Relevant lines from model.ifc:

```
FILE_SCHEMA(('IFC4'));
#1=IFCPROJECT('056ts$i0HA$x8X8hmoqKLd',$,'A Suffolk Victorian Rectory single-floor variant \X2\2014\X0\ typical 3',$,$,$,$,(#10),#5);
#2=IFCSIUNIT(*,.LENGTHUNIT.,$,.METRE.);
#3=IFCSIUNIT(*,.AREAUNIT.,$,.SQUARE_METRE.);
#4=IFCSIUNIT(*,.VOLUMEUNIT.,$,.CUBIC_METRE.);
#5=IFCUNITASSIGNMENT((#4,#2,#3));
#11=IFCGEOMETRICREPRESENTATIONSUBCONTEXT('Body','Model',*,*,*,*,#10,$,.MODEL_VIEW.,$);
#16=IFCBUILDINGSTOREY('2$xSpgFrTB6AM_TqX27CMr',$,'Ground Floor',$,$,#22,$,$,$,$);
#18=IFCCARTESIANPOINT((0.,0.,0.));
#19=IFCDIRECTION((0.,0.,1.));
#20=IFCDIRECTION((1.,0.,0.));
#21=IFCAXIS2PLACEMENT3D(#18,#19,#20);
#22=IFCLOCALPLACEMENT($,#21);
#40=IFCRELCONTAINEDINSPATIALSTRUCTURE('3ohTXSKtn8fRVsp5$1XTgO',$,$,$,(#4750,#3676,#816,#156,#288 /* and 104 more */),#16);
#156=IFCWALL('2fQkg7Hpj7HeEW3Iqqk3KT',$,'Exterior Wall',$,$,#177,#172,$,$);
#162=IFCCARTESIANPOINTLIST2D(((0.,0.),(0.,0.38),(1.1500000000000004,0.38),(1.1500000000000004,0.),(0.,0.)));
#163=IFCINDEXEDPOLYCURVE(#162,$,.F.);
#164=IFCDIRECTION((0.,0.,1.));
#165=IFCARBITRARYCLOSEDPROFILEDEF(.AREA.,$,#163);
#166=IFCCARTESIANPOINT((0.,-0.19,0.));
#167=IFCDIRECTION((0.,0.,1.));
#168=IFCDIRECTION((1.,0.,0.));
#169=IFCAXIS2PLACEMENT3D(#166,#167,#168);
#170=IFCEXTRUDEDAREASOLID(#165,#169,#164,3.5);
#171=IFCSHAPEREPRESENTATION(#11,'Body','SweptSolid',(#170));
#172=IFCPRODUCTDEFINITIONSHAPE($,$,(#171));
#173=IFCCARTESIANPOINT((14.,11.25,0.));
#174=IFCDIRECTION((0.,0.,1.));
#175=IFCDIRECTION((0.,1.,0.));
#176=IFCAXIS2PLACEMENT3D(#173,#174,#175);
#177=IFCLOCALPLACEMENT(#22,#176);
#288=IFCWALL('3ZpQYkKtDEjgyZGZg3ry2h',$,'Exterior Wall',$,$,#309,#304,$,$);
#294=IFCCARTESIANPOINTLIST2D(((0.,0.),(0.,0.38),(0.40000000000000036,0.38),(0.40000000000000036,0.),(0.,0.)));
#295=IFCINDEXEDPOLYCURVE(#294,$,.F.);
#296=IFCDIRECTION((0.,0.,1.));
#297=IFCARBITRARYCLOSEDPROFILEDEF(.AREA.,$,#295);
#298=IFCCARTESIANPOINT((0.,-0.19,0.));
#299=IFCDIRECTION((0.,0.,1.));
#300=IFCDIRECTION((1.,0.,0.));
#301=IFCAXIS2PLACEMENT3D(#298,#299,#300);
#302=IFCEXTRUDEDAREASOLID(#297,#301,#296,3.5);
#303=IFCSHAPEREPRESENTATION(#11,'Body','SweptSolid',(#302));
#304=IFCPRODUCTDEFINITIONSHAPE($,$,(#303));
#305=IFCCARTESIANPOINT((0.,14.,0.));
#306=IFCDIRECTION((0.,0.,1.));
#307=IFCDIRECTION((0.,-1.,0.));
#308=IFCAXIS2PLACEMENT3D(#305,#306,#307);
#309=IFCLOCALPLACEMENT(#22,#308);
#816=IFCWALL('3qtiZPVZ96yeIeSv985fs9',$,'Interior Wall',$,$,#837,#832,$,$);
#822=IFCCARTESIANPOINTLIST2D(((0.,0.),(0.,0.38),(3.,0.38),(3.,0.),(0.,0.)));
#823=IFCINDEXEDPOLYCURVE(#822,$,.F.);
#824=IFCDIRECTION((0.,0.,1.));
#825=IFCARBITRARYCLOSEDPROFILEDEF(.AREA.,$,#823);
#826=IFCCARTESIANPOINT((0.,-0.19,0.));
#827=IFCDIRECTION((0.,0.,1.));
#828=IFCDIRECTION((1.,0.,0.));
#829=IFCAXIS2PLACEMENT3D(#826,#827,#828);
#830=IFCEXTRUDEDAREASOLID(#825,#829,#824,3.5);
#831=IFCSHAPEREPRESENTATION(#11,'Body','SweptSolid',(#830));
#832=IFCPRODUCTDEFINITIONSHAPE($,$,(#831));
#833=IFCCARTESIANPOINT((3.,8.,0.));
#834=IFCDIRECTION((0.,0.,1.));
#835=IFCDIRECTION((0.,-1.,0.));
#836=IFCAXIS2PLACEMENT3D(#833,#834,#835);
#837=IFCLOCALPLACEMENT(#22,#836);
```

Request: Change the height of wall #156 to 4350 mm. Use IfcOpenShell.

```python
import ifcopenshell
import ifcopenshell.geom
import ifcopenshell.util.representation
import ifcopenshell.util.shape

model = ifcopenshell.open("model.ifc")
settings = ifcopenshell.geom.settings()


def volume(element):
    """Net volume in cubic metres, openings subtracted."""
    shape = ifcopenshell.geom.create_shape(settings, element)
    return ifcopenshell.util.shape.get_volume(shape.geometry)


wall = model.by_guid("2fQkg7Hpj7HeEW3Iqqk3KT")
before = volume(wall)

body = ifcopenshell.util.representation.get_representation(wall, "Model", "Body")
solid = body.Items[0]
old_height = solid.Depth
solid.Depth = 4.35
after = volume(wall)

print(f"height {old_height:g} -> {solid.Depth:g}, volume {before:.3f} -> {after:.3f} m3")

model.write("model-out.ifc")
```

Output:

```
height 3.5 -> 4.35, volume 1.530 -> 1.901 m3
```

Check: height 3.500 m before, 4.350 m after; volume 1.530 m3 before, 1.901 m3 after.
